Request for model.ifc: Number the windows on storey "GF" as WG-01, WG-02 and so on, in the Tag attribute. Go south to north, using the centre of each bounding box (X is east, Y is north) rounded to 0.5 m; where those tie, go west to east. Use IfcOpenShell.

First a look at what the model holds.

```python
import ifcopenshell
import ifcopenshell.util.element
import ifcopenshell.util.placement

model = ifcopenshell.open("model.ifc")
print(model.schema)
storey = next(s for s in model.by_type("IfcBuildingStorey") if s.Name == "GF")
windows = [e for e in ifcopenshell.util.element.get_decomposition(storey) if e.is_a("IfcWindow")]
for e in sorted(windows, key=lambda e: e.id()):
    origin = ifcopenshell.util.placement.get_local_placement(e.ObjectPlacement)[:3, 3]
    print(e.id(), e.Tag, e.Name, origin.round(2) + 0.0, sep=" | ")
```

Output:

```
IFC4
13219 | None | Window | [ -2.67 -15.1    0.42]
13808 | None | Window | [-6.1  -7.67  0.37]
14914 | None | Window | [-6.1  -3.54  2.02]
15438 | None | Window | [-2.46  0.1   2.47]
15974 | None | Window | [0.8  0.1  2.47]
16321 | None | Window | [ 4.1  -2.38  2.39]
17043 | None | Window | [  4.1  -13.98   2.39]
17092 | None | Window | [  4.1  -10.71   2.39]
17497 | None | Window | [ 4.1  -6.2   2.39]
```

```python
import ifcopenshell
import ifcopenshell.geom
import ifcopenshell.util.element
import ifcopenshell.util.shape

model = ifcopenshell.open("model.ifc")
settings = ifcopenshell.geom.settings()
settings.set("use-world-coords", True)


def centre(element):
    shape = ifcopenshell.geom.create_shape(settings, element)
    return ifcopenshell.util.shape.get_bbox_centroid(shape.geometry)


storey = next(s for s in model.by_type("IfcBuildingStorey") if s.Name == "GF")
windows = [e for e in ifcopenshell.util.element.get_decomposition(storey) if e.is_a("IfcWindow")]

# Insertion points can sit at a corner or the storey origin, so sort by the geometry (in metres).
centres = {e: centre(e) for e in windows}
windows.sort(key=lambda e: (round(centres[e][1] / 0.5), centres[e][0]))

for i, e in enumerate(windows, start=1):
    number = f"WG-{i:02d}"
    e.Tag = number
    print(e.id(), number)

model.write("model-out.ifc")
```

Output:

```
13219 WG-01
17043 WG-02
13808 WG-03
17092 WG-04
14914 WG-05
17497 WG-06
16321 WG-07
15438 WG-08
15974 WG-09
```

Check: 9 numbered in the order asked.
